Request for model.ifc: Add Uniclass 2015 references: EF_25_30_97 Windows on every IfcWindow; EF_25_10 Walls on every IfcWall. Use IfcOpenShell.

First a look at what the model holds.

```python
import ifcopenshell

model = ifcopenshell.open("model.ifc")
print(model.schema)
print("classifications:", [c.Name for c in model.by_type("IfcClassification")])
for ifc_class in ("IfcDoor", "IfcRoof", "IfcStair", "IfcWall", "IfcWindow"):
    print(ifc_class, len(model.by_type(ifc_class)))
```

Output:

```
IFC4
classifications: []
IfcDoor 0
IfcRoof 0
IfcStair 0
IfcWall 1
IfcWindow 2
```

```python
import ifcopenshell
import ifcopenshell.api.classification

model = ifcopenshell.open("model.ifc")

system = ifcopenshell.api.classification.add_classification(model, classification="Uniclass 2015")

codes = {
    "IfcWindow": ("EF_25_30_97", "Windows"),
    "IfcWall": ("EF_25_10", "Walls"),
}
for ifc_class, (code, name) in codes.items():
    products = model.by_type(ifc_class)
    ifcopenshell.api.classification.add_reference(
        model, products=products, classification=system, identification=code, name=name
    )
    print(code, len(products))

model.write("model_rev.ifc")
```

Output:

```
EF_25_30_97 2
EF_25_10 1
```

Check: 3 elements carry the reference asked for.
